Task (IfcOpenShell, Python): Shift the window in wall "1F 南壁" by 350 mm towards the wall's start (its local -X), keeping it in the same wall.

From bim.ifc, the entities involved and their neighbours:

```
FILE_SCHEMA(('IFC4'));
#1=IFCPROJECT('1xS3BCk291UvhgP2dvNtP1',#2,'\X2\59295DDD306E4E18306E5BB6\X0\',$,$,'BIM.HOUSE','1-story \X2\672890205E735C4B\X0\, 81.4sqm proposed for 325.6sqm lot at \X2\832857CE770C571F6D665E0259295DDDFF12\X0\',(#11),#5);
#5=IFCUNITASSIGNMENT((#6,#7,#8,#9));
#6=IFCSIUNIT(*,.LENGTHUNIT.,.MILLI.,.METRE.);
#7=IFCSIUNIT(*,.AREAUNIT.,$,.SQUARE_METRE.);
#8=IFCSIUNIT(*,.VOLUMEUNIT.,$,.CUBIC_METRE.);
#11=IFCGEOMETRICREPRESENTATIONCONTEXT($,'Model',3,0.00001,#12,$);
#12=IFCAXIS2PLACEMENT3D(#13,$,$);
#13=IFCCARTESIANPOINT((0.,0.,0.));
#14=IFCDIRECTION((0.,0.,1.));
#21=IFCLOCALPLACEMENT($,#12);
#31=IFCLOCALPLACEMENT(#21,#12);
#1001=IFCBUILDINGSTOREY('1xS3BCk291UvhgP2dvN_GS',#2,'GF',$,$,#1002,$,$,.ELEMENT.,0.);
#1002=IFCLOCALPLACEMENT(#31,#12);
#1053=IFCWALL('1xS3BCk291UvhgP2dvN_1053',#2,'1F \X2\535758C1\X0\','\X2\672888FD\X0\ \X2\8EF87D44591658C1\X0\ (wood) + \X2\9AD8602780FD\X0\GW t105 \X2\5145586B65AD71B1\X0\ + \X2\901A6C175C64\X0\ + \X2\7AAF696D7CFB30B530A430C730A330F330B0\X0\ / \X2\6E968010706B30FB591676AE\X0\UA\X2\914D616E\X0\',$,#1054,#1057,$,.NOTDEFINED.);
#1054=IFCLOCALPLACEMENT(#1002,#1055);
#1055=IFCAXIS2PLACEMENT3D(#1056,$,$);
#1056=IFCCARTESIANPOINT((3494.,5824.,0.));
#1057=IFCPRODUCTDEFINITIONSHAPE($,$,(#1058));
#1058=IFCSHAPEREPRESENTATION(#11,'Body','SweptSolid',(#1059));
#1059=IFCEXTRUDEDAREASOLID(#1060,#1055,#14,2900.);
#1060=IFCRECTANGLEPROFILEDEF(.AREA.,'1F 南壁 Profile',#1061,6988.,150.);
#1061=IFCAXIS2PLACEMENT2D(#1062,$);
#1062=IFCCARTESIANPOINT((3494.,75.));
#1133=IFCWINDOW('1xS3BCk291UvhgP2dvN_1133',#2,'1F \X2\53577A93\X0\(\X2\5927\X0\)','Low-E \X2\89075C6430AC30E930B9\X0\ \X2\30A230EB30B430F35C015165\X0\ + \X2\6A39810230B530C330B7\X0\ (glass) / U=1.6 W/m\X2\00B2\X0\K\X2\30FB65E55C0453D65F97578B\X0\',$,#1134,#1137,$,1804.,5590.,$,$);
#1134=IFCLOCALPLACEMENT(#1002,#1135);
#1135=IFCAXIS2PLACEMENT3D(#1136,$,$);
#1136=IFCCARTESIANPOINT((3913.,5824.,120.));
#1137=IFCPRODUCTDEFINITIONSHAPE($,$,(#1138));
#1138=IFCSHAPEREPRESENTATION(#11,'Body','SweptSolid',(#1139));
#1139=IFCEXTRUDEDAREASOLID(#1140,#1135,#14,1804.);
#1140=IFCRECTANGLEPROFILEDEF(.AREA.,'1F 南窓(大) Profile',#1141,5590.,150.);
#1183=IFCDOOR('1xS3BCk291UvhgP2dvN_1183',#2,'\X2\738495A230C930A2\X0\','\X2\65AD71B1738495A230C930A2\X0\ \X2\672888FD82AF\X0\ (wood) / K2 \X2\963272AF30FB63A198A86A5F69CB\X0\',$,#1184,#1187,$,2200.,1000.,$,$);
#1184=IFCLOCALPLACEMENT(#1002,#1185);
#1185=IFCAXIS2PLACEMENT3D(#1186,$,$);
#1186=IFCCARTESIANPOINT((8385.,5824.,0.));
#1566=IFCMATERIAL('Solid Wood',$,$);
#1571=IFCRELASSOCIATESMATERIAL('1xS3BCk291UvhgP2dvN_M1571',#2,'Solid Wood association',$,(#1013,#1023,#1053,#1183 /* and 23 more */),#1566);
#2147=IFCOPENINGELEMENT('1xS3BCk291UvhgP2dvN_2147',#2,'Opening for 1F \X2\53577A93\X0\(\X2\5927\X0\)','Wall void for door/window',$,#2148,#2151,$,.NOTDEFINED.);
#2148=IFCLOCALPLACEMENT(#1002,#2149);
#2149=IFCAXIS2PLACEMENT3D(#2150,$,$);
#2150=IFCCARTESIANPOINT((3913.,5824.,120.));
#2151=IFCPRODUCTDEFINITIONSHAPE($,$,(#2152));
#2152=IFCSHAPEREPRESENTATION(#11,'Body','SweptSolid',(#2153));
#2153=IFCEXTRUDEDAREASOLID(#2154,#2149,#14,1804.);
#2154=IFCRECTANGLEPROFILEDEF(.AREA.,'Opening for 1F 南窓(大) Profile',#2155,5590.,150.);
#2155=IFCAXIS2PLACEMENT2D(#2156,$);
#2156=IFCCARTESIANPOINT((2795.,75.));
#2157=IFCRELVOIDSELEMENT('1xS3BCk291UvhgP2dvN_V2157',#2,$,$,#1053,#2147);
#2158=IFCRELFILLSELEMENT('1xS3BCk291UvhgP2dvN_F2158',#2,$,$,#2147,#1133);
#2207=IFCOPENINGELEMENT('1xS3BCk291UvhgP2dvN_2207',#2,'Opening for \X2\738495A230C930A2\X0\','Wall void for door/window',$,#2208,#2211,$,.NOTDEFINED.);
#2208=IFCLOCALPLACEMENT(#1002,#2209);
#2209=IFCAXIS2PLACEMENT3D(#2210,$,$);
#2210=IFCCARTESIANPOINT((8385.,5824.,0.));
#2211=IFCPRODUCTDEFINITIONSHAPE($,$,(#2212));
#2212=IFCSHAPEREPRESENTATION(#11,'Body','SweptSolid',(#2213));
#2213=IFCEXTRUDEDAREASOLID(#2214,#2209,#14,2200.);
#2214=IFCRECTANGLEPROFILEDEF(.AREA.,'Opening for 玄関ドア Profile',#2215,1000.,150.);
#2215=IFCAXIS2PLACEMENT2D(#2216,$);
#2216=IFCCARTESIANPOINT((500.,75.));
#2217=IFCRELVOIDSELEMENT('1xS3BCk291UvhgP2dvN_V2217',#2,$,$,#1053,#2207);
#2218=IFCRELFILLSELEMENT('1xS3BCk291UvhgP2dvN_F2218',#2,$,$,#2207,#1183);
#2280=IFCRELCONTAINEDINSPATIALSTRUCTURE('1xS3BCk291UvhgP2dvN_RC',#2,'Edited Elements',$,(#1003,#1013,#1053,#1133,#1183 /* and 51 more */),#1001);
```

```python
import ifcopenshell
import ifcopenshell.api.geometry
import ifcopenshell.util.placement
import ifcopenshell.util.unit

model = ifcopenshell.open("bim.ifc")
unit_scale = ifcopenshell.util.unit.calculate_unit_scale(model)

window = model.by_guid("1xS3BCk291UvhgP2dvN_1133")
opening = window.FillsVoids[0].RelatingOpeningElement
wall = opening.VoidsElements[0].RelatingBuildingElement

wall_matrix = ifcopenshell.util.placement.get_local_placement(wall.ObjectPlacement)
shift = wall_matrix[:3, 0] * -0.35 / unit_scale
before = ifcopenshell.util.placement.get_local_placement(window.ObjectPlacement)[:3, 3].copy()

# The window is not placed relative to its opening, so move both.
for product in (opening, window):
    matrix = ifcopenshell.util.placement.get_local_placement(product.ObjectPlacement)
    matrix[:3, 3] += shift
    ifcopenshell.api.geometry.edit_object_placement(model, product=product, matrix=matrix, is_si=False)

after = ifcopenshell.util.placement.get_local_placement(window.ObjectPlacement)[:3, 3]
print("window moved by", (after - before).round(3) + 0.0)

model.write("bim-out.ifc")
```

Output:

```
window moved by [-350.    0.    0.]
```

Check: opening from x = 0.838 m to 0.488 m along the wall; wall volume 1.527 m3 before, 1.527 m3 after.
